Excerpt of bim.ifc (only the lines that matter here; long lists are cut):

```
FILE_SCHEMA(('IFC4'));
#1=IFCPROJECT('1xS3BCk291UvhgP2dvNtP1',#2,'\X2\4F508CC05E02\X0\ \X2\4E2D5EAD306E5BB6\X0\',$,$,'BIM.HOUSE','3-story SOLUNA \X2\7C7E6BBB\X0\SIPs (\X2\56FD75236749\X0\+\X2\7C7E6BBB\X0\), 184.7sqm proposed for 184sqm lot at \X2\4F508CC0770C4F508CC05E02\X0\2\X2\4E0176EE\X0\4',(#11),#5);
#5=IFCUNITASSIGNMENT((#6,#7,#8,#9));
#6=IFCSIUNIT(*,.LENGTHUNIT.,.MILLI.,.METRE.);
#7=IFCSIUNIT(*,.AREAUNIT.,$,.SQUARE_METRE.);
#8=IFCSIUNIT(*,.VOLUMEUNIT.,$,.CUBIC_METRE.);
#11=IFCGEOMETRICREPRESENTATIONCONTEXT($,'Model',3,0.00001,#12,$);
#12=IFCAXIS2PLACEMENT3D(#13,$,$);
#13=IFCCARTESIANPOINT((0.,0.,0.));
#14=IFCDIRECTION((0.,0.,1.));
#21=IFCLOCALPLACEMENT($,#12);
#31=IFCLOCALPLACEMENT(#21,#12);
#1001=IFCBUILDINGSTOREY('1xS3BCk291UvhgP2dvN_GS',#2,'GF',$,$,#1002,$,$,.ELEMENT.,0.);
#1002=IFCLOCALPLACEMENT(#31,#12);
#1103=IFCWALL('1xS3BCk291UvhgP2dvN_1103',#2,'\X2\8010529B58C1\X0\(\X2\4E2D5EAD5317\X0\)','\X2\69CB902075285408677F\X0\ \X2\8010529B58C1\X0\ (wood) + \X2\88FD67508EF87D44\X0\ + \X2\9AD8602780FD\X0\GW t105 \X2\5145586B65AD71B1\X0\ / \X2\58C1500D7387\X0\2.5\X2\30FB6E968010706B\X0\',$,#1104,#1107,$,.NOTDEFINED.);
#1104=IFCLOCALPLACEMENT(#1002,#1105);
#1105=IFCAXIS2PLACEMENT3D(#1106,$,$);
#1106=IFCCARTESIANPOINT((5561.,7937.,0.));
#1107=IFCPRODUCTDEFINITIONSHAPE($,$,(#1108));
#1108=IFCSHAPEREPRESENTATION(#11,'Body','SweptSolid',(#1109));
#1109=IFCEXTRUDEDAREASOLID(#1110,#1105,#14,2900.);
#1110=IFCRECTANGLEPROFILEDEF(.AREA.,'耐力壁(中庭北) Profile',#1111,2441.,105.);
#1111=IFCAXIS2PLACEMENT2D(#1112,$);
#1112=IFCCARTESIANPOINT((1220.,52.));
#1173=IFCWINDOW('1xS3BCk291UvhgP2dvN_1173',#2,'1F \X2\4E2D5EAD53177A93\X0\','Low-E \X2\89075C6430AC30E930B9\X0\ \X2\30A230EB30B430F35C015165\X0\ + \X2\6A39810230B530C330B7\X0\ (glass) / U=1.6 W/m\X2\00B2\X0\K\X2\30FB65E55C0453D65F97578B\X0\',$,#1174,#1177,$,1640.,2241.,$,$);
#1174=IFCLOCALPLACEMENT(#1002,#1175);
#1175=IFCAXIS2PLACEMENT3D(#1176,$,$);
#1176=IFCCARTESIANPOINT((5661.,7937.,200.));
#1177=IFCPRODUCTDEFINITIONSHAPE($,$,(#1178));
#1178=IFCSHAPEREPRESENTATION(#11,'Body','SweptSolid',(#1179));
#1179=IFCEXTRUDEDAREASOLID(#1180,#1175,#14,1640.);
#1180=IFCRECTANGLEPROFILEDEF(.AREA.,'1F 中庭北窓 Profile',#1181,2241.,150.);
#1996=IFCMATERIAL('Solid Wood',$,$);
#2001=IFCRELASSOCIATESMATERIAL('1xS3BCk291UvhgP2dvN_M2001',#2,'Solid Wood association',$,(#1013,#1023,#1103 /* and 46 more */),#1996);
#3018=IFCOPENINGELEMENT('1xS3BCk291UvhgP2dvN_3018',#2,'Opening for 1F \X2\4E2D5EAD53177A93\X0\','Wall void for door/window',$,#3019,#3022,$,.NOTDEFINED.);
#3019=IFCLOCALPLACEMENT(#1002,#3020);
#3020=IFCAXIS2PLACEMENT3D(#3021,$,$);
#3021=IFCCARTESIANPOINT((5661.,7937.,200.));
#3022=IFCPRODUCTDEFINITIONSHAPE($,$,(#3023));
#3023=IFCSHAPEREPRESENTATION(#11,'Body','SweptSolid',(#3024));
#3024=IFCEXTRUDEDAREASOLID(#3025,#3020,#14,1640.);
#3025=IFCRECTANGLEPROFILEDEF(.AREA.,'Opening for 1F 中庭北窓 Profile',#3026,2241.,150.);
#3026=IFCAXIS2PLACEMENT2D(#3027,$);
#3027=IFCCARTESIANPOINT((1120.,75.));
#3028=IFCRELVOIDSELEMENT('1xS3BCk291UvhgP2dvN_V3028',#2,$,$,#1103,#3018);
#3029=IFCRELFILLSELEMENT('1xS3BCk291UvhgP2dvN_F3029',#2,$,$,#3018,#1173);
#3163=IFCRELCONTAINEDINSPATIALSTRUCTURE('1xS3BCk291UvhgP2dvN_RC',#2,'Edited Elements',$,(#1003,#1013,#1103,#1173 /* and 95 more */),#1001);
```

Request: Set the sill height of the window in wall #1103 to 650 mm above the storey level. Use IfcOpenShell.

```python
import numpy as np
import ifcopenshell
import ifcopenshell.api.geometry
import ifcopenshell.geom
import ifcopenshell.util.element
import ifcopenshell.util.placement
import ifcopenshell.util.shape
import ifcopenshell.util.unit

model = ifcopenshell.open("bim.ifc")
unit_scale = ifcopenshell.util.unit.calculate_unit_scale(model)

window = model.by_guid("1xS3BCk291UvhgP2dvN_1173")
opening = window.FillsVoids[0].RelatingOpeningElement
storey = ifcopenshell.util.element.get_container(window, ifc_class="IfcBuildingStorey")
level = ifcopenshell.util.placement.get_local_placement(storey.ObjectPlacement)[2, 3]

# The opening's origin need not be at the sill, so measure its lowest point.
shape = ifcopenshell.geom.create_shape(ifcopenshell.geom.settings(), opening)
bottom = ifcopenshell.util.shape.get_shape_bottom_elevation(shape, shape.geometry) / unit_scale
dz = level + 650.0 - bottom

shift = np.array([0.0, 0.0, dz])
# The window is not placed relative to its opening, so move both.
for product in (opening, window):
    matrix = ifcopenshell.util.placement.get_local_placement(product.ObjectPlacement)
    matrix[:3, 3] += shift
    ifcopenshell.api.geometry.edit_object_placement(model, product=product, matrix=matrix, is_si=False)

print(f"moved by {dz * unit_scale:+.3f} m")

model.write("bim_rev.ifc")
```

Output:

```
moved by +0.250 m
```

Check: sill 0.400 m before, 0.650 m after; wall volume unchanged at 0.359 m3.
